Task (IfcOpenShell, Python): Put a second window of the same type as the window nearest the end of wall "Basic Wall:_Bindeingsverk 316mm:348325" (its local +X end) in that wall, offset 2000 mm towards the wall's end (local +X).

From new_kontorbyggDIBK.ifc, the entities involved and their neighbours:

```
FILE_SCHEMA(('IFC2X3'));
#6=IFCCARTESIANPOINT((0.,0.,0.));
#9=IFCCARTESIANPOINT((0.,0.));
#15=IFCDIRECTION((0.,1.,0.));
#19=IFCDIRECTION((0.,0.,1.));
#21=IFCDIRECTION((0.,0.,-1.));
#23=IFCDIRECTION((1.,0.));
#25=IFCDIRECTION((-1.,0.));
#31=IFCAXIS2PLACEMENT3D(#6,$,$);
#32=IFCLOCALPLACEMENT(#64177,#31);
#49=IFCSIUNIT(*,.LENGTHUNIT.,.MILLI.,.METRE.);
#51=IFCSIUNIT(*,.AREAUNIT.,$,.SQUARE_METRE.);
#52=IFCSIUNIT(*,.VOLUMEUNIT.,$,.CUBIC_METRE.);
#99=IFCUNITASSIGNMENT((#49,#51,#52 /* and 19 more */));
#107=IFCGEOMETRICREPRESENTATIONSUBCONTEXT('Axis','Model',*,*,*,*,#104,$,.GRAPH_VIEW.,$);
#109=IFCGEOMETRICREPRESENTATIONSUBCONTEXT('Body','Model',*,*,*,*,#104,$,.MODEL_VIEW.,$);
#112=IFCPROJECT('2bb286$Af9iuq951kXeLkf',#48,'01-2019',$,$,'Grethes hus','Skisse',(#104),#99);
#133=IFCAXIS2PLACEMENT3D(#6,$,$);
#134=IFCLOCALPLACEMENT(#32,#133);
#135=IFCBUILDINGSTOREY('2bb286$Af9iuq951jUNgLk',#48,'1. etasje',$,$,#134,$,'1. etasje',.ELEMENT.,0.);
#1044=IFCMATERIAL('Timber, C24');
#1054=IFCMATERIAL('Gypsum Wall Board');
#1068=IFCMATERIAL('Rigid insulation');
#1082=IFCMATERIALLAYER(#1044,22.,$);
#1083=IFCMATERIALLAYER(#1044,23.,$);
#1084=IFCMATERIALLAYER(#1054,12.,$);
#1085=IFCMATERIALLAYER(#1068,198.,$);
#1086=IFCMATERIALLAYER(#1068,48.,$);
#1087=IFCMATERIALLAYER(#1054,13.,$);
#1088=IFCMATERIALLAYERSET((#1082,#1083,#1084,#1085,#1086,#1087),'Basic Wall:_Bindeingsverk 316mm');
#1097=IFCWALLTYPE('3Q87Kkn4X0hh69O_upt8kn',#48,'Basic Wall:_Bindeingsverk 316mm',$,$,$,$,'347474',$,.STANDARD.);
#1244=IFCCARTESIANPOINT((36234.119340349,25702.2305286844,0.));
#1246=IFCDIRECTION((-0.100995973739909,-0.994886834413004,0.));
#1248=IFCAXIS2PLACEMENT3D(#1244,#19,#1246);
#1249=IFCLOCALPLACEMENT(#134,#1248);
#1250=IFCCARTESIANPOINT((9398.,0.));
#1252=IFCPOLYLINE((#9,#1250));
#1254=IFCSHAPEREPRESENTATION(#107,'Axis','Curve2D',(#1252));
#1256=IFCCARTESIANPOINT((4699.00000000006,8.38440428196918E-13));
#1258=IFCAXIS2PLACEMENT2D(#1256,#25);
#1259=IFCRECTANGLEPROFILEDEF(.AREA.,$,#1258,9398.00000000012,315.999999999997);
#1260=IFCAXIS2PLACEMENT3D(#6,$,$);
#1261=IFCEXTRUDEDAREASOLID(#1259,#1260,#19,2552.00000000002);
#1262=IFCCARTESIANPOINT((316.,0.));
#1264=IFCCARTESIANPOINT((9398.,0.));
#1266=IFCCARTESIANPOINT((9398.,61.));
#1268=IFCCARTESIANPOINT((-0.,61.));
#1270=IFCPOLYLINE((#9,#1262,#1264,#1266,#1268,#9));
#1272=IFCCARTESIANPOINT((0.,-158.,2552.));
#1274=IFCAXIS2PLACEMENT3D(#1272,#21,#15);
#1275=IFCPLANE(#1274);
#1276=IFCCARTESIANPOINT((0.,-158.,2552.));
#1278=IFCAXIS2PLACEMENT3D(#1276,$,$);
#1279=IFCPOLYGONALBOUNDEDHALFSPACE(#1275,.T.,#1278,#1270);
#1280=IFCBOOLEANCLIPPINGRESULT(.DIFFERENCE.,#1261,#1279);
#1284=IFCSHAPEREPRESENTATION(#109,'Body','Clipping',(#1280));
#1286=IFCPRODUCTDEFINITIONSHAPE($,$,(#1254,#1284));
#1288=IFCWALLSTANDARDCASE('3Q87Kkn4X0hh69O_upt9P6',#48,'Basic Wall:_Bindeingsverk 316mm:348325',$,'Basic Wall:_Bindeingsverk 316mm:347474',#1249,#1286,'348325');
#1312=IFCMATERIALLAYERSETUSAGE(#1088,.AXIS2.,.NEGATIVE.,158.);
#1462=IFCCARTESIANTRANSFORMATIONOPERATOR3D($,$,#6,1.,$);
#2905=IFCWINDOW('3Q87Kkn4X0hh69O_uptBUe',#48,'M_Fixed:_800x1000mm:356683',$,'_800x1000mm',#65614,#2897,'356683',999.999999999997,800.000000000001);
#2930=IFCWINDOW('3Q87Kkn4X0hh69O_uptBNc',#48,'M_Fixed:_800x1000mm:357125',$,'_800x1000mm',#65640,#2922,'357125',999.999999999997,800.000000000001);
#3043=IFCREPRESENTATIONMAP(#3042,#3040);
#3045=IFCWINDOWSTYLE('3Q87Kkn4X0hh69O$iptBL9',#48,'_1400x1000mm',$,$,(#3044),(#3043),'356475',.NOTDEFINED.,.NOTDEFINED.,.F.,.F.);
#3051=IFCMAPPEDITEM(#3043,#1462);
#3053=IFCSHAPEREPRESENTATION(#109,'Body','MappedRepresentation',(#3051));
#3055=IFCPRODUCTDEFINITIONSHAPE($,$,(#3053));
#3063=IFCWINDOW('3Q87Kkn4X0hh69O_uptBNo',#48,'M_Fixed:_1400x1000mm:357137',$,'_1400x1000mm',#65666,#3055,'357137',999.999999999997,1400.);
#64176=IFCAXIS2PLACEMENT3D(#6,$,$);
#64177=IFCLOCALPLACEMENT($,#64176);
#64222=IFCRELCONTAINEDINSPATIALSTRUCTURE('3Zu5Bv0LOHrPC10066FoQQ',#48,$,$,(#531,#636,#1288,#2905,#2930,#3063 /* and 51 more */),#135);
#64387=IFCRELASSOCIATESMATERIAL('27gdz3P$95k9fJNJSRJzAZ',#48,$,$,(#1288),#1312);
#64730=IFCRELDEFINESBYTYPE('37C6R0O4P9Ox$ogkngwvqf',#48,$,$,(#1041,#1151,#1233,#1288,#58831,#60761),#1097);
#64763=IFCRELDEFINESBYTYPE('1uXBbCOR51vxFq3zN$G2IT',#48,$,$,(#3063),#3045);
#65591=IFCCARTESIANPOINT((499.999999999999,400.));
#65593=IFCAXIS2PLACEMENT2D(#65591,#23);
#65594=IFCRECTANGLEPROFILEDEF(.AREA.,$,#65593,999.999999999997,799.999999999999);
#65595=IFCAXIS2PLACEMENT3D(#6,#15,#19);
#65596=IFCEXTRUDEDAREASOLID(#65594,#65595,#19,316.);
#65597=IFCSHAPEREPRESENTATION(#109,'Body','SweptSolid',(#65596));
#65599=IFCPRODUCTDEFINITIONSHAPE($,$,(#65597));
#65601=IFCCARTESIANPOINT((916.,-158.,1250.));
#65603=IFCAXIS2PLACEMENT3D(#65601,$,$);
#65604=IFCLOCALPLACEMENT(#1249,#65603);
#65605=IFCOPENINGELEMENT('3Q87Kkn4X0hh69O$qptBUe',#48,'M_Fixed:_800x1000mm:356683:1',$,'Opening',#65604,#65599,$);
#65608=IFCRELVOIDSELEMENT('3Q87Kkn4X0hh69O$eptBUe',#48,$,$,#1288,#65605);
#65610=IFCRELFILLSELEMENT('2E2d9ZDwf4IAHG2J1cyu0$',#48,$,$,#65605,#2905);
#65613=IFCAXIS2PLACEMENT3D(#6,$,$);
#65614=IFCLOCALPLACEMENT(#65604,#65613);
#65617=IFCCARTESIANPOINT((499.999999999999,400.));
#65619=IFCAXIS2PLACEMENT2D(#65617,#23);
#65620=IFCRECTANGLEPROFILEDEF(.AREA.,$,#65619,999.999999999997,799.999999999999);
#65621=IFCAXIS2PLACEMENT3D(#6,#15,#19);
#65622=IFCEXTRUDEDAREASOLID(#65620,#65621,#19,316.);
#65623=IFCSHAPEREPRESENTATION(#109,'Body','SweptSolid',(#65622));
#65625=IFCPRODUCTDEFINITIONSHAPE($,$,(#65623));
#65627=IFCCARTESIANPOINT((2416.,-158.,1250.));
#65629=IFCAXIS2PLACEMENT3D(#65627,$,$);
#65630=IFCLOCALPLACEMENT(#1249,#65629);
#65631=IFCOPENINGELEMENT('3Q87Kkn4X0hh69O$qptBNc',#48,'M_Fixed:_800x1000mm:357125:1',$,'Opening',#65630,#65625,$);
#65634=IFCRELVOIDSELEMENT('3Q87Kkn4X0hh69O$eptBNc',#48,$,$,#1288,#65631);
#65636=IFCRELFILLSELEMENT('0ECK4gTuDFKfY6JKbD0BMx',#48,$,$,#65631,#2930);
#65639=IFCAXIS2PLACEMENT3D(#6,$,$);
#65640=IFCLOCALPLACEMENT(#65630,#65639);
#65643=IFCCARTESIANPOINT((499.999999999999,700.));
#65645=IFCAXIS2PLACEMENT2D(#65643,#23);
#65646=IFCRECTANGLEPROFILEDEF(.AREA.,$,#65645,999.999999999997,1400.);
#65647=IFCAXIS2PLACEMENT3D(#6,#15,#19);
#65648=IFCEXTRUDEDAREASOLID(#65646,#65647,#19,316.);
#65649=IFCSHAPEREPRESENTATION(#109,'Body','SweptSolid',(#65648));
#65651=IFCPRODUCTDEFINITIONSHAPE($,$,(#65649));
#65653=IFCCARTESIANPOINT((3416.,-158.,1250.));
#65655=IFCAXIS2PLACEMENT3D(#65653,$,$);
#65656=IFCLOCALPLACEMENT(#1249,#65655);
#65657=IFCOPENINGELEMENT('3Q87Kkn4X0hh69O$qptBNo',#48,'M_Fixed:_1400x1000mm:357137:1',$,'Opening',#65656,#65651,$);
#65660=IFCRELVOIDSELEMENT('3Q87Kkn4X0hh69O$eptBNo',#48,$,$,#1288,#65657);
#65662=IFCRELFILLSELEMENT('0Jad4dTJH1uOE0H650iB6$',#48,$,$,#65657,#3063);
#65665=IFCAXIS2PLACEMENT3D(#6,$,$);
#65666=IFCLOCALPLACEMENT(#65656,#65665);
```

```python
import ifcopenshell
import ifcopenshell.api.feature
import ifcopenshell.api.geometry
import ifcopenshell.api.root
import ifcopenshell.geom
import ifcopenshell.util.element
import ifcopenshell.util.placement
import ifcopenshell.util.shape
import ifcopenshell.util.unit

model = ifcopenshell.open("new_kontorbyggDIBK.ifc")
unit_scale = ifcopenshell.util.unit.calculate_unit_scale(model)
settings = ifcopenshell.geom.settings()


def volume(element):
    """Net volume in cubic metres, openings subtracted."""
    shape = ifcopenshell.geom.create_shape(settings, element)
    return ifcopenshell.util.shape.get_volume(shape.geometry)


def reuse_history(source, copy):
    """copy_class also copies each property set's owner history, people and application; keep the originals."""
    for rel in copy.IsDefinedBy:
        if rel.is_a("IfcRelDefinesByProperties") and (history := rel.RelatingPropertyDefinition.OwnerHistory):
            rel.RelatingPropertyDefinition.OwnerHistory = source.OwnerHistory
            ifcopenshell.util.element.remove_deep2(model, history)


window = model.by_id(3063)
opening = window.FillsVoids[0].RelatingOpeningElement
wall = opening.VoidsElements[0].RelatingBuildingElement
before = volume(wall)
shift = ifcopenshell.util.placement.get_local_placement(wall.ObjectPlacement)[:3, 0] * 2 / unit_scale

# copy_class copies the void relationship, type, container and properties, but no geometry.
new_opening = ifcopenshell.api.root.copy_class(model, product=opening)
new_opening.Representation = ifcopenshell.util.element.copy_deep(
    model, opening.Representation, exclude=["IfcGeometricRepresentationContext", "IfcRepresentationMap"]
)
new_opening.Name = "M_Fixed:_1400x1000mm"
new_window = ifcopenshell.api.root.copy_class(model, product=window)
new_window.Representation = ifcopenshell.util.element.copy_deep(
    model, window.Representation, exclude=["IfcGeometricRepresentationContext", "IfcRepresentationMap"]
)
new_window.Name = "M_Fixed:_1400x1000mm"
new_window.Tag = None
reuse_history(window, new_window)
fills = ifcopenshell.api.feature.add_filling(model, opening=new_opening, element=new_window)
fills.OwnerHistory = new_window.OwnerHistory  # required in IFC2X3

for old, new in ((opening, new_opening), (window, new_window)):
    matrix = ifcopenshell.util.placement.get_local_placement(old.ObjectPlacement)
    matrix[:3, 3] += shift
    ifcopenshell.api.geometry.edit_object_placement(model, product=new, matrix=matrix, is_si=False)

after = volume(wall)

print(f"wall volume {before:.3f} -> {after:.3f} m3")

model.write("new_kontorbyggDIBK_v2.ifc")
```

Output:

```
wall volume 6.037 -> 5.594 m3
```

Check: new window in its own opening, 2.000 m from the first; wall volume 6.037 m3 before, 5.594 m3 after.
